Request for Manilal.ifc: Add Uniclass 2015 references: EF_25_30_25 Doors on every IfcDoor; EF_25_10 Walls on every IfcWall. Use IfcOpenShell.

First a look at what the model holds.

```python
import ifcopenshell

model = ifcopenshell.open("Manilal.ifc")
print(model.schema)
print("classifications:", [c.Name for c in model.by_type("IfcClassification")])
for ifc_class in ("IfcDoor", "IfcRoof", "IfcStair", "IfcWall", "IfcWindow"):
    print(ifc_class, len(model.by_type(ifc_class)))
```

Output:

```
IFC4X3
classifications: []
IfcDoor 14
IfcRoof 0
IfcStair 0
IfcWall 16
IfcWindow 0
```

```python
import ifcopenshell
import ifcopenshell.api.classification

model = ifcopenshell.open("Manilal.ifc")

system = ifcopenshell.api.classification.add_classification(model, classification="Uniclass 2015")

codes = {
    "IfcDoor": ("EF_25_30_25", "Doors"),
    "IfcWall": ("EF_25_10", "Walls"),
}
for ifc_class, (code, name) in codes.items():
    products = model.by_type(ifc_class)
    ifcopenshell.api.classification.add_reference(
        model, products=products, classification=system, identification=code, name=name
    )
    print(code, len(products))

model.write("Manilal_edited.ifc")
```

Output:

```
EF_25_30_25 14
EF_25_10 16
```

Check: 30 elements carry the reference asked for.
